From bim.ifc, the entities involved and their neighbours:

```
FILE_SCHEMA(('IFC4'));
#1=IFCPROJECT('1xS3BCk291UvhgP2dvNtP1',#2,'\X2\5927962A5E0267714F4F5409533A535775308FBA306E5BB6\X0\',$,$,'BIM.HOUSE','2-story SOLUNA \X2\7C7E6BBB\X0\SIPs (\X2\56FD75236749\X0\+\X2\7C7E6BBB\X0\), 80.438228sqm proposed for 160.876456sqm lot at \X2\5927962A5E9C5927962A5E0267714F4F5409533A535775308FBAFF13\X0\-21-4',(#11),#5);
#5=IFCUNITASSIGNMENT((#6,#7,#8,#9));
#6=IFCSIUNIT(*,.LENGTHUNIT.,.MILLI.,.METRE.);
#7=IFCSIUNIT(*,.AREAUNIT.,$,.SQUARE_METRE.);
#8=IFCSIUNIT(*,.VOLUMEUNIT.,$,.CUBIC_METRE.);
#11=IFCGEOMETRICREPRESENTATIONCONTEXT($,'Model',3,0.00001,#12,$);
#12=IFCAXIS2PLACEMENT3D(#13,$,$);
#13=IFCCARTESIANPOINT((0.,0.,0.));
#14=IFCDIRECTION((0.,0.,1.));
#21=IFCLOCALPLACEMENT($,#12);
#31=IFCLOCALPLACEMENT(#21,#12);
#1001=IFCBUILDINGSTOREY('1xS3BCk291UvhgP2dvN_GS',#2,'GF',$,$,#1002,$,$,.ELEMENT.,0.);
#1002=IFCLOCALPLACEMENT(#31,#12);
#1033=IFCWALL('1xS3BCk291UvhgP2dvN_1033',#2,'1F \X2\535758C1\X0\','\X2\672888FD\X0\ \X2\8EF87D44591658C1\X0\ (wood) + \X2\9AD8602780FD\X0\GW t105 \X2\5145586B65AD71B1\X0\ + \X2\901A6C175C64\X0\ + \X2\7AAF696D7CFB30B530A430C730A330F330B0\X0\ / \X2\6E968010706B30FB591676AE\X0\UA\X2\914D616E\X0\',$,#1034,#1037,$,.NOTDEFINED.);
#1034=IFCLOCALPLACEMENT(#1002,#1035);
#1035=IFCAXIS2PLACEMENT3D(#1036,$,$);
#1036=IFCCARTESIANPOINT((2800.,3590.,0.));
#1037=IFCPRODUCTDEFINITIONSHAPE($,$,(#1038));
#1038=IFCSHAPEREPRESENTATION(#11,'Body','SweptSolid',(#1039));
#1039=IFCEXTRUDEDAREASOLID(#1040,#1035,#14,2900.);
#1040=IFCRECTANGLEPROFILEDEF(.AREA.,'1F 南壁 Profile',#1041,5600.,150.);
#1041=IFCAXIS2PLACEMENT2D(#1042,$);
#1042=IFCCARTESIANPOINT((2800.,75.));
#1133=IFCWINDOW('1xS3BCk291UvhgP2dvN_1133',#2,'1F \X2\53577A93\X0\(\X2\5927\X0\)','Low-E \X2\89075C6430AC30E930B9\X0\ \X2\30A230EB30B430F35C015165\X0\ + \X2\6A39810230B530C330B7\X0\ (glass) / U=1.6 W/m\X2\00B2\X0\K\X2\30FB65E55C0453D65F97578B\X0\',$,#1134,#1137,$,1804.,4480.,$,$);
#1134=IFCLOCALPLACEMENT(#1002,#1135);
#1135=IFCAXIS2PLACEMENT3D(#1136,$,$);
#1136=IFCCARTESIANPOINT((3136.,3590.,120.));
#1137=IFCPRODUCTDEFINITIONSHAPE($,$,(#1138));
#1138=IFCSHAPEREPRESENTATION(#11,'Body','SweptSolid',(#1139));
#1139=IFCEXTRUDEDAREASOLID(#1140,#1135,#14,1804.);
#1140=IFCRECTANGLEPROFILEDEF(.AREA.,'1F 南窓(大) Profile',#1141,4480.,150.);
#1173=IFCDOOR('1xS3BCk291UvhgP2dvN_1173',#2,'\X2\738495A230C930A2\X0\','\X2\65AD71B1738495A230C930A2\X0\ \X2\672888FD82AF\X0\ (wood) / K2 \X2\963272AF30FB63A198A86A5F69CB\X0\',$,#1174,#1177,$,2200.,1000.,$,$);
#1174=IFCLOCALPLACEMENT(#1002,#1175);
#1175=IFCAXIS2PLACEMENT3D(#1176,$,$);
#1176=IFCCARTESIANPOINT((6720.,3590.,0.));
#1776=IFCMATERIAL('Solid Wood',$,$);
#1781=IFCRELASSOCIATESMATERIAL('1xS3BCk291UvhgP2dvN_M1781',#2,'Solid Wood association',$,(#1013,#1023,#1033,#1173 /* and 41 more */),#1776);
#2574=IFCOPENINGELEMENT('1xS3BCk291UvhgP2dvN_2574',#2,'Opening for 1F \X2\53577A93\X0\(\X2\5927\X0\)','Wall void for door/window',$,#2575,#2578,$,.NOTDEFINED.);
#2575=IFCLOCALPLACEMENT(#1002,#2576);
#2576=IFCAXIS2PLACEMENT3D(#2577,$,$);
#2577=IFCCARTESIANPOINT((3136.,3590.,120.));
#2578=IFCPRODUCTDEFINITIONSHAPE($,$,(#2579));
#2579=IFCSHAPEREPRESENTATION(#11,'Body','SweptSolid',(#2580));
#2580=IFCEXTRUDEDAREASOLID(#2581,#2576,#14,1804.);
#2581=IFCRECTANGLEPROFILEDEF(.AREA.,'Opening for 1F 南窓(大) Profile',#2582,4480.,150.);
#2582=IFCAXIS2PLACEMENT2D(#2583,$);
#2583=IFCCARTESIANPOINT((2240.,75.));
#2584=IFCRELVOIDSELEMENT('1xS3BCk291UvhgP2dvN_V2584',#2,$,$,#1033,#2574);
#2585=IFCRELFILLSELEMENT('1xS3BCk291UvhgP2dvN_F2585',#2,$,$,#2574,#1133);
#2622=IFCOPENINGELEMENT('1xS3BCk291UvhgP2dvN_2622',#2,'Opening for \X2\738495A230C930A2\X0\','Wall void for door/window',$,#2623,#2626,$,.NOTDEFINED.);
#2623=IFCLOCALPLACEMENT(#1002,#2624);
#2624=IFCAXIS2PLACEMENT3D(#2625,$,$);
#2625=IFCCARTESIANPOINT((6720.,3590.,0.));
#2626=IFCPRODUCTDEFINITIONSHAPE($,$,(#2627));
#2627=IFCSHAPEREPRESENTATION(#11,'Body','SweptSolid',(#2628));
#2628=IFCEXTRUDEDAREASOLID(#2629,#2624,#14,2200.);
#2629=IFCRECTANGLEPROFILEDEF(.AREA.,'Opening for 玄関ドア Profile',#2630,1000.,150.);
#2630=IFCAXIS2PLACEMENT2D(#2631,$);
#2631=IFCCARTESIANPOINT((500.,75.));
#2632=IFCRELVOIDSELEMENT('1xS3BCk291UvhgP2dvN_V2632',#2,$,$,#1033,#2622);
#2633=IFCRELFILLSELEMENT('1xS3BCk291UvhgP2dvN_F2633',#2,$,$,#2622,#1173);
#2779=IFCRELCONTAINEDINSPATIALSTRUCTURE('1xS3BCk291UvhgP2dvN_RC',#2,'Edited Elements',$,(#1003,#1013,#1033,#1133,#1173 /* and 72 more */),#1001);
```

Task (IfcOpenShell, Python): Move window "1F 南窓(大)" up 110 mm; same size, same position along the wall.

```python
import numpy as np
import ifcopenshell
import ifcopenshell.api.geometry
import ifcopenshell.util.placement
import ifcopenshell.util.unit

model = ifcopenshell.open("bim.ifc")
unit_scale = ifcopenshell.util.unit.calculate_unit_scale(model)

window = model.by_id(1133)
opening = window.FillsVoids[0].RelatingOpeningElement
dz = 110.0

shift = np.array([0.0, 0.0, dz])
# The window is not placed relative to its opening, so move both.
for product in (opening, window):
    matrix = ifcopenshell.util.placement.get_local_placement(product.ObjectPlacement)
    matrix[:3, 3] += shift
    ifcopenshell.api.geometry.edit_object_placement(model, product=product, matrix=matrix, is_si=False)

print(f"moved by {dz * unit_scale:+.3f} m")

model.write("bim-out.ifc")
```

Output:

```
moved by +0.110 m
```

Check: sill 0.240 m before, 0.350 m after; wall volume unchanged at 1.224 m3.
